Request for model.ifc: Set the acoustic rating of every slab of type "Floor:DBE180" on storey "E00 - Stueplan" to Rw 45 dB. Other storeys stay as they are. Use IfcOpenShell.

First a look at what the model holds.

```python
import ifcopenshell
import ifcopenshell.util.element

model = ifcopenshell.open("model.ifc")
print(model.schema)
storey = next(s for s in model.by_type("IfcBuildingStorey") if s.Name == "E00 - Stueplan")
slabs = [e for e in ifcopenshell.util.element.get_decomposition(storey) if e.is_a("IfcSlab")]
seen = {}
for e in slabs:
    element_type = ifcopenshell.util.element.get_type(e)
    key = (element_type.Name if element_type != e and element_type else None, ifcopenshell.util.element.get_pset(e, "Pset_SlabCommon", "AcousticRating"))
    seen[key] = seen.get(key, 0) + 1
for (name, value), count in sorted(seen.items(), key=str):
    print(count, "x", name, "|", value)
```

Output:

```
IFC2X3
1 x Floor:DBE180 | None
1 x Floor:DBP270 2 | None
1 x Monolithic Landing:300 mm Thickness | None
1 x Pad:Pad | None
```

```python
import ifcopenshell
import ifcopenshell.api.pset
import ifcopenshell.util.element

model = ifcopenshell.open("model.ifc")

storey = next(s for s in model.by_type("IfcBuildingStorey") if s.Name == "E00 - Stueplan")
slabs = [e for e in ifcopenshell.util.element.get_decomposition(storey) if e.is_a("IfcSlab")]

count = 0
for e in slabs:
    element_type = ifcopenshell.util.element.get_type(e)
    if element_type in (None, e) or element_type.Name != "Floor:DBE180":
        continue
    # add_pset returns the element's existing set when there is one.
    pset = ifcopenshell.api.pset.add_pset(model, product=e, name="Pset_SlabCommon")
    ifcopenshell.api.pset.edit_pset(model, pset=pset, properties={"AcousticRating": "Rw 45 dB"})
    count += 1

print(count, "slabs updated")

model.write("model_updated.ifc")
```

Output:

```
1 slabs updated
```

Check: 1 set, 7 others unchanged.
